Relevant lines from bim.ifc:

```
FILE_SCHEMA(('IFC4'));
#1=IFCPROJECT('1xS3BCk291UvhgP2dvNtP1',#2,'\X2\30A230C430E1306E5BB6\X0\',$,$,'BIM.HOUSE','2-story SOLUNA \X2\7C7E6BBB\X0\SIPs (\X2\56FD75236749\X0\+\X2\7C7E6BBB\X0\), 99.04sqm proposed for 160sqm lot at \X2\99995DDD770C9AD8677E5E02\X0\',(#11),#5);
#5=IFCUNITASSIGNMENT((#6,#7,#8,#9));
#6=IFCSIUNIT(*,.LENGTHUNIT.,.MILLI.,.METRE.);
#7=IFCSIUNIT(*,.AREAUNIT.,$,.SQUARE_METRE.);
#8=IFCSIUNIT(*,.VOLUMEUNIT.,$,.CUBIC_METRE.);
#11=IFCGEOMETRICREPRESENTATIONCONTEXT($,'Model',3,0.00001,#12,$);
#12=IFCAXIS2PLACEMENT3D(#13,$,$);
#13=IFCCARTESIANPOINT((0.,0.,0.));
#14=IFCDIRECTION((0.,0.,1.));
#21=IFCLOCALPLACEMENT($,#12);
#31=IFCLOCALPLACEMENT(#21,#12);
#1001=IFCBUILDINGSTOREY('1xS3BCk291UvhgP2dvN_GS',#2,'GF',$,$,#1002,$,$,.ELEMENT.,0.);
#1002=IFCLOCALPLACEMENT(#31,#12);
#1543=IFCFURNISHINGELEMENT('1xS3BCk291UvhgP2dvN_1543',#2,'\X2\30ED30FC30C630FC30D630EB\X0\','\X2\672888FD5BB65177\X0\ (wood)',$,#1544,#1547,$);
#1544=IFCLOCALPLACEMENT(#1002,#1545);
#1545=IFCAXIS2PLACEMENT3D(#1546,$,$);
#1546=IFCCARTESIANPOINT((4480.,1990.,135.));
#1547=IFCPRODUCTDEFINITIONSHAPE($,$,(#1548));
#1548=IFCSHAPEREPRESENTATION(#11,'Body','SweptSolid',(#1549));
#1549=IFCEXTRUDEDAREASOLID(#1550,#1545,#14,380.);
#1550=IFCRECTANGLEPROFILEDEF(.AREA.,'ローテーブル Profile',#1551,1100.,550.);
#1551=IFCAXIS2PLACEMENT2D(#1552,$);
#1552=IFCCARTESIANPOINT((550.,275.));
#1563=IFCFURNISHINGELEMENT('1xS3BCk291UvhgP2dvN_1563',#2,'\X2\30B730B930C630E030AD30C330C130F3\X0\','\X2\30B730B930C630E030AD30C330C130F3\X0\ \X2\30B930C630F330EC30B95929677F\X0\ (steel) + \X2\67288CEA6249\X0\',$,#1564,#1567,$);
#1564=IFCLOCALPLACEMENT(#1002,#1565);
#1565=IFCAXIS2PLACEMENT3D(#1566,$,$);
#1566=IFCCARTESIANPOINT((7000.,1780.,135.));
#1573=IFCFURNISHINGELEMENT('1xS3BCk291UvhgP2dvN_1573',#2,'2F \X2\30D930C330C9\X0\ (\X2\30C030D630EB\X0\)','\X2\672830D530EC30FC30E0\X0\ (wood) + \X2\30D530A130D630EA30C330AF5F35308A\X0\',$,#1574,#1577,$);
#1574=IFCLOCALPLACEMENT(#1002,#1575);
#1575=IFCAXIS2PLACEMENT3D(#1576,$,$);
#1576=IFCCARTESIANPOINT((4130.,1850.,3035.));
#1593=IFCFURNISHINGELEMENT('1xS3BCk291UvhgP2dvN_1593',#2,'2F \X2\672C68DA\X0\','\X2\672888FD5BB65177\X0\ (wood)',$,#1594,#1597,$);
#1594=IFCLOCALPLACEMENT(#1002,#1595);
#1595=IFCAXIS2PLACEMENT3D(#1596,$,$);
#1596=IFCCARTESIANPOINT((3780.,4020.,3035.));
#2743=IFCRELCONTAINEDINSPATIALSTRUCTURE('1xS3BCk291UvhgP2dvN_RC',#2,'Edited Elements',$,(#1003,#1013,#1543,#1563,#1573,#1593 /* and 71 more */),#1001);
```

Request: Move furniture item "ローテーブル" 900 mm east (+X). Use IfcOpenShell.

```python
import ifcopenshell
import ifcopenshell.api.geometry
import ifcopenshell.util.placement
import ifcopenshell.util.unit

model = ifcopenshell.open("bim.ifc")
unit_scale = ifcopenshell.util.unit.calculate_unit_scale(model)

item = model.by_guid("1xS3BCk291UvhgP2dvN_1543")
matrix = ifcopenshell.util.placement.get_local_placement(item.ObjectPlacement)
matrix[0, 3] += 0.9 / unit_scale
ifcopenshell.api.geometry.edit_object_placement(model, product=item, matrix=matrix, is_si=False)

print(ifcopenshell.util.placement.get_local_placement(item.ObjectPlacement).round(3) + 0.0)

model.write("bim_rev.ifc")
```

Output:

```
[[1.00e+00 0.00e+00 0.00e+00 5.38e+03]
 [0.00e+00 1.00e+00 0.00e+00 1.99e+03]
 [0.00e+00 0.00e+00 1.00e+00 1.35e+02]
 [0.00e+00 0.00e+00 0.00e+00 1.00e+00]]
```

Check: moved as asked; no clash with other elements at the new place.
